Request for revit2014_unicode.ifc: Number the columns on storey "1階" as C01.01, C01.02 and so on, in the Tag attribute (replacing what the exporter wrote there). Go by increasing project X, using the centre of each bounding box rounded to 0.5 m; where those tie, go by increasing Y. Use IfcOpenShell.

First a look at what the model holds.

```python
import ifcopenshell
import ifcopenshell.util.element
import ifcopenshell.util.placement

model = ifcopenshell.open("revit2014_unicode.ifc")
print(model.schema)
storey = next(s for s in model.by_type("IfcBuildingStorey") if s.Name == "1階")
columns = [e for e in ifcopenshell.util.element.get_decomposition(storey) if e.is_a("IfcColumn")]
for e in sorted(columns, key=lambda e: e.id()):
    origin = ifcopenshell.util.placement.get_local_placement(e.ObjectPlacement)[:3, 3]
    print(e.id(), e.Tag, e.Name, origin.round(2) + 0.0, sep=" | ")
```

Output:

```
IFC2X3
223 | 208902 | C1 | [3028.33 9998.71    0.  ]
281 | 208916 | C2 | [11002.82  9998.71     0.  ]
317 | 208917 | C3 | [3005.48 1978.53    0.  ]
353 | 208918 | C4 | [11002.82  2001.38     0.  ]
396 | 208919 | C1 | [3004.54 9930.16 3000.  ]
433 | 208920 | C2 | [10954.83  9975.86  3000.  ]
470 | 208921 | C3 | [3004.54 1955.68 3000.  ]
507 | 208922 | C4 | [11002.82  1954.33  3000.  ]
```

```python
import ifcopenshell
import ifcopenshell.geom
import ifcopenshell.util.element
import ifcopenshell.util.shape

model = ifcopenshell.open("revit2014_unicode.ifc")
settings = ifcopenshell.geom.settings()
settings.set("use-world-coords", True)


def centre(element):
    shape = ifcopenshell.geom.create_shape(settings, element)
    return ifcopenshell.util.shape.get_bbox_centroid(shape.geometry)


storey = next(s for s in model.by_type("IfcBuildingStorey") if s.Name == "1階")
columns = [e for e in ifcopenshell.util.element.get_decomposition(storey) if e.is_a("IfcColumn")]

# Insertion points can sit at a corner or the storey origin, so sort by the geometry (in metres).
centres = {e: centre(e) for e in columns}
columns.sort(key=lambda e: (round(centres[e][0] / 0.5), centres[e][1]))

for i, e in enumerate(columns, start=1):
    number = f"C01.{i:02d}"
    e.Tag = number
    print(e.id(), number)

model.write("revit2014_unicode-out.ifc")
```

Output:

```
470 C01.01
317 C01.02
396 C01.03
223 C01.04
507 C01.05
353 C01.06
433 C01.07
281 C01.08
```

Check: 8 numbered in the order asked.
